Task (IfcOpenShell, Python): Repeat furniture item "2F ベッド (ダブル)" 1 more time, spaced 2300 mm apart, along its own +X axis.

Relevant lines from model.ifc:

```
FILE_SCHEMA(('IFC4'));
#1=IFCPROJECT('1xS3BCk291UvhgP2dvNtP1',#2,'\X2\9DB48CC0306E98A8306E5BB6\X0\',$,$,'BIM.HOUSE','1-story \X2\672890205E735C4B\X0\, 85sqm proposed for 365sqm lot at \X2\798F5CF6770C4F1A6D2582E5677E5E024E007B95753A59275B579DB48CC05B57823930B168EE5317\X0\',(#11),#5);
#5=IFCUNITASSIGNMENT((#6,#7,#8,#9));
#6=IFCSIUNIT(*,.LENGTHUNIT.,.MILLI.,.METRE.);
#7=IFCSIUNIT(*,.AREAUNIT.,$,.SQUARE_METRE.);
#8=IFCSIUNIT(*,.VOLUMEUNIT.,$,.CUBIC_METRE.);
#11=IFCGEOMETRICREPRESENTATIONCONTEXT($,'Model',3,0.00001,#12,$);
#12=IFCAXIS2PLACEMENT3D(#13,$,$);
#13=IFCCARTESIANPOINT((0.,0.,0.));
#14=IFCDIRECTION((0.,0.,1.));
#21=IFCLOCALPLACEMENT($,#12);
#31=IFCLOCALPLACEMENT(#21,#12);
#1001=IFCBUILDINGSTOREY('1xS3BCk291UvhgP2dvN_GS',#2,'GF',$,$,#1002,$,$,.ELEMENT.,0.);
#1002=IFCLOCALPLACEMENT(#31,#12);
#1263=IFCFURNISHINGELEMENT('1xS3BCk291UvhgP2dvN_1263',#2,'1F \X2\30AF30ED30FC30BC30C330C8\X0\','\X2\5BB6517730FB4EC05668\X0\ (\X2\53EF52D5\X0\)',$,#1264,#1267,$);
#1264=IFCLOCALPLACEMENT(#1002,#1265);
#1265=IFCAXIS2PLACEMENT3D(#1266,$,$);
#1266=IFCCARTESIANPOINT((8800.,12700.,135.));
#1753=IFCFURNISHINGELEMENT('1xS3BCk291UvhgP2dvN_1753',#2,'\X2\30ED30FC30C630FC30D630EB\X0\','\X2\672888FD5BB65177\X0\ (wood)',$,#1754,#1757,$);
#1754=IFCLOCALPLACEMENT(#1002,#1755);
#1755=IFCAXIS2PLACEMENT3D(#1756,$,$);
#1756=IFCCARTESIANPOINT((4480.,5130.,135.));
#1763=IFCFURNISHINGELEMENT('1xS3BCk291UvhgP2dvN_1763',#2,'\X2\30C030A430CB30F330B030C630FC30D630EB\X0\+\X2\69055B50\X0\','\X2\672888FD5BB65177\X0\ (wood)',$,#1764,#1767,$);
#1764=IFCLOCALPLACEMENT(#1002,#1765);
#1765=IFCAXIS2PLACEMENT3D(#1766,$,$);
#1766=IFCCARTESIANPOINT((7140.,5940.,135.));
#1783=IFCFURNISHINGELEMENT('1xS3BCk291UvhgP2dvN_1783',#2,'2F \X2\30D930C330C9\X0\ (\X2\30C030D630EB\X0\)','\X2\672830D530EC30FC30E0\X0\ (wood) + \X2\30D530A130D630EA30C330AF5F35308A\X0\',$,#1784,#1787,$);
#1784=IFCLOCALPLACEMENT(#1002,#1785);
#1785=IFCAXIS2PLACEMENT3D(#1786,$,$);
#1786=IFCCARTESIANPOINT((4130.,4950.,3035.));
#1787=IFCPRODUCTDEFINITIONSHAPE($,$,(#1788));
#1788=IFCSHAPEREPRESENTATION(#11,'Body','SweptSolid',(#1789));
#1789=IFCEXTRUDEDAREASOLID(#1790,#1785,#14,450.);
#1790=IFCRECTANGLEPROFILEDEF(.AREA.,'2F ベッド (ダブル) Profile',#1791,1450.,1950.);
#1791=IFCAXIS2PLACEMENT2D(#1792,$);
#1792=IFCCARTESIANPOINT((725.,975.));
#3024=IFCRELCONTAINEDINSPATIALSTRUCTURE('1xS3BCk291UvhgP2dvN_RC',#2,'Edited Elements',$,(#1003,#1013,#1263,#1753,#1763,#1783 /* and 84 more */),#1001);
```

```python
import ifcopenshell
import ifcopenshell.api.geometry
import ifcopenshell.api.root
import ifcopenshell.util.element
import ifcopenshell.util.placement

model = ifcopenshell.open("model.ifc")


def reuse_history(source, copy):
    """copy_class also copies each property set's owner history, people and application; keep the originals."""
    for rel in copy.IsDefinedBy:
        if rel.is_a("IfcRelDefinesByProperties") and (history := rel.RelatingPropertyDefinition.OwnerHistory):
            rel.RelatingPropertyDefinition.OwnerHistory = source.OwnerHistory
            ifcopenshell.util.element.remove_deep2(model, history)


source = model.by_id(1783)
base = ifcopenshell.util.placement.get_local_placement(source.ObjectPlacement)
step = base[:3, 0] * 2300.0

for i in range(1, 2):
    copy = ifcopenshell.api.root.copy_class(model, product=source)
    copy.Representation = ifcopenshell.util.element.copy_deep(
        model, source.Representation, exclude=["IfcGeometricRepresentationContext", "IfcRepresentationMap"]
    )
    reuse_history(source, copy)
    matrix = base.copy()
    matrix[:3, 3] += i * step
    print("added at", matrix[:3, 3].round(3) + 0.0)
    ifcopenshell.api.geometry.edit_object_placement(model, product=copy, matrix=matrix, is_si=False)

model.write("model_rev.ifc")
```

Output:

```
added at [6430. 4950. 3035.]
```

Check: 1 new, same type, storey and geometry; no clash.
